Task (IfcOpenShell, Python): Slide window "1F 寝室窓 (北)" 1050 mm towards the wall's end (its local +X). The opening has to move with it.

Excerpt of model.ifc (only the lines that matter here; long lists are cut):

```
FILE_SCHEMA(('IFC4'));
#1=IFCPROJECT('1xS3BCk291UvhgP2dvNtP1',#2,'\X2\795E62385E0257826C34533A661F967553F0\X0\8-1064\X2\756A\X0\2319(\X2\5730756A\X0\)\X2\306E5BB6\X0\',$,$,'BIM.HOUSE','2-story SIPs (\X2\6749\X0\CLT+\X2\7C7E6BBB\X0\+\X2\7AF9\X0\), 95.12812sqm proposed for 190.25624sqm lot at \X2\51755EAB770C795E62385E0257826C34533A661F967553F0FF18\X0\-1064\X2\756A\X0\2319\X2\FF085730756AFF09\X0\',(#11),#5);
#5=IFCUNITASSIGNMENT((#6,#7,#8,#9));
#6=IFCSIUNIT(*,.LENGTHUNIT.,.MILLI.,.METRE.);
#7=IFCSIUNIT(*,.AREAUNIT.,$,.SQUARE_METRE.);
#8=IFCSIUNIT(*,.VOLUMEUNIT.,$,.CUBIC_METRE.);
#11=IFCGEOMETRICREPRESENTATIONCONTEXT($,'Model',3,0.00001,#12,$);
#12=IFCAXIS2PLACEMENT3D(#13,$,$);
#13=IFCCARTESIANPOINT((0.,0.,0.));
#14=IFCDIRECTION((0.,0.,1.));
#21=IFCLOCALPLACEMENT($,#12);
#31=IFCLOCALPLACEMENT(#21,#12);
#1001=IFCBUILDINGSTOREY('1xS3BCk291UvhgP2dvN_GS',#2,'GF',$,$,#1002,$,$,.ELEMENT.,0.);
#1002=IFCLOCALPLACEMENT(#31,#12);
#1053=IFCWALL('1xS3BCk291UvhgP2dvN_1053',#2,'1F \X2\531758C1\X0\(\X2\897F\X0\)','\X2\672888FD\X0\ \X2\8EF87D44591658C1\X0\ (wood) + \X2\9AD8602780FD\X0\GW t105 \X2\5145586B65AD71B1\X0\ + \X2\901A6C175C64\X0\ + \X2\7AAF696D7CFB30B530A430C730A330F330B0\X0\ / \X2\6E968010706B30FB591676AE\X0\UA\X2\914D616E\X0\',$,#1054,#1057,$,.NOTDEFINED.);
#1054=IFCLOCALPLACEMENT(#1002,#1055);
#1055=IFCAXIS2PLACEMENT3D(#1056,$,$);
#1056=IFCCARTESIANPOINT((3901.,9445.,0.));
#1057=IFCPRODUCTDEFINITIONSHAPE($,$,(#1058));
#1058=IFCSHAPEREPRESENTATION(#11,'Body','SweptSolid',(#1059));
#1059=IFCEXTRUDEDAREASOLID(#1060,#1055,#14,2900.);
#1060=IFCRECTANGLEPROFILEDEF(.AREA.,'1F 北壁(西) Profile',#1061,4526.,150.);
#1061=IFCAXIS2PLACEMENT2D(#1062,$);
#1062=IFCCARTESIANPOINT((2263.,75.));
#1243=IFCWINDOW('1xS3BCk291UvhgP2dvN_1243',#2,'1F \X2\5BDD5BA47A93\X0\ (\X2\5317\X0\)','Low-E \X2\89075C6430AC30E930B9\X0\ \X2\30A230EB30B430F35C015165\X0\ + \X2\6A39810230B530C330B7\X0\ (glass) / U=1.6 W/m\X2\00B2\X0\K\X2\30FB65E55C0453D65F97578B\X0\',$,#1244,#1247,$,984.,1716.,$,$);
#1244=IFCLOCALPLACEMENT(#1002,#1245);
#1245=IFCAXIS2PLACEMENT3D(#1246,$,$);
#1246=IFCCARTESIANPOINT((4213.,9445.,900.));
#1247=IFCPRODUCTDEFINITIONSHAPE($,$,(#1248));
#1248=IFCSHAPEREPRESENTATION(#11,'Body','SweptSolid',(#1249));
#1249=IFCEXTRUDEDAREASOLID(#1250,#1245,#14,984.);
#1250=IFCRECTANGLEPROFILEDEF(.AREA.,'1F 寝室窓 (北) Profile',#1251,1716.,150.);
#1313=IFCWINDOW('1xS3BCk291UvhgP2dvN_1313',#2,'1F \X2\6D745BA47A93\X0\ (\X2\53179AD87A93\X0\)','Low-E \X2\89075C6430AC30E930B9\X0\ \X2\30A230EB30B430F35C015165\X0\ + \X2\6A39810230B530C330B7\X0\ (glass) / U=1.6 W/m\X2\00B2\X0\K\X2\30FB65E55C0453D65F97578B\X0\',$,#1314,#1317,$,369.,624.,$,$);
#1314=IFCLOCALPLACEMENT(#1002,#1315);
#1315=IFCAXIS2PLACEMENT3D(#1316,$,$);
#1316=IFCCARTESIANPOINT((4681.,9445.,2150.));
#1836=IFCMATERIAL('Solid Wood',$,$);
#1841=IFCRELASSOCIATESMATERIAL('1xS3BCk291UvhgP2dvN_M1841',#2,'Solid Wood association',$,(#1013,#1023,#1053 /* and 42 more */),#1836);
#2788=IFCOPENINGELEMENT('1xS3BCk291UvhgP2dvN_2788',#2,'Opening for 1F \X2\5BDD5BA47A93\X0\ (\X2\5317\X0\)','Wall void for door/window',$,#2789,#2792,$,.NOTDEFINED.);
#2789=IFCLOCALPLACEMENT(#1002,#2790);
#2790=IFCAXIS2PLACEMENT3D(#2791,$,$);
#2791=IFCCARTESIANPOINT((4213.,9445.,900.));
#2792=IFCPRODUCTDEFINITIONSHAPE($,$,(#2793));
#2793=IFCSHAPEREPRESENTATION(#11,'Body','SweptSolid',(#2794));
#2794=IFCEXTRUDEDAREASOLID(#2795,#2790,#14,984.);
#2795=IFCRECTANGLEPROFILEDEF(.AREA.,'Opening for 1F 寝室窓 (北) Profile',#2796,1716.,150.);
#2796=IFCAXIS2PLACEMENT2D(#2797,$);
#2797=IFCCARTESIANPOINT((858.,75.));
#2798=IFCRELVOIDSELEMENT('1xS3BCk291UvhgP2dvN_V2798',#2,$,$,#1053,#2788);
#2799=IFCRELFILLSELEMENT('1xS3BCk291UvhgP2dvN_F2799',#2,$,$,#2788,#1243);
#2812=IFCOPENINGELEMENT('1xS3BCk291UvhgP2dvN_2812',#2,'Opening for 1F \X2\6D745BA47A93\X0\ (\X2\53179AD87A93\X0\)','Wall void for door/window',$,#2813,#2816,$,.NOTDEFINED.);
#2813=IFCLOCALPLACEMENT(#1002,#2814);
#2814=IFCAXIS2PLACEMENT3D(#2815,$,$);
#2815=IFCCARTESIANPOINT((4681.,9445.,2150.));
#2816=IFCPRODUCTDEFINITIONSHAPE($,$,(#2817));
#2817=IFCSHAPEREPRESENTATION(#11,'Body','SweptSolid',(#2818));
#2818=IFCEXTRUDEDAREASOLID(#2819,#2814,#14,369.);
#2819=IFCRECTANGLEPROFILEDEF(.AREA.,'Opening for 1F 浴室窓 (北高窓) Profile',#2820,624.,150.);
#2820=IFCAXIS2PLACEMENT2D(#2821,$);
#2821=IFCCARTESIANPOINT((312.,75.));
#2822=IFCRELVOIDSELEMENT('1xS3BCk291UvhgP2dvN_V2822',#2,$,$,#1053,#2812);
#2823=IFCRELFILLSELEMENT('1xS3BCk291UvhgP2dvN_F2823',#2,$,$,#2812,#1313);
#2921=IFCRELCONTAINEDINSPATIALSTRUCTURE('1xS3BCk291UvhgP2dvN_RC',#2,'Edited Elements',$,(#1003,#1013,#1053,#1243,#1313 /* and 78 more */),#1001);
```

```python
import ifcopenshell
import ifcopenshell.api.geometry
import ifcopenshell.util.placement
import ifcopenshell.util.unit

model = ifcopenshell.open("model.ifc")
unit_scale = ifcopenshell.util.unit.calculate_unit_scale(model)

window = model.by_guid("1xS3BCk291UvhgP2dvN_1243")
opening = window.FillsVoids[0].RelatingOpeningElement
wall = opening.VoidsElements[0].RelatingBuildingElement

wall_matrix = ifcopenshell.util.placement.get_local_placement(wall.ObjectPlacement)
shift = wall_matrix[:3, 0] * 1.05 / unit_scale
before = ifcopenshell.util.placement.get_local_placement(window.ObjectPlacement)[:3, 3].copy()

# The window is not placed relative to its opening, so move both.
for product in (opening, window):
    matrix = ifcopenshell.util.placement.get_local_placement(product.ObjectPlacement)
    matrix[:3, 3] += shift
    ifcopenshell.api.geometry.edit_object_placement(model, product=product, matrix=matrix, is_si=False)

after = ifcopenshell.util.placement.get_local_placement(window.ObjectPlacement)[:3, 3]
print("window moved by", (after - before).round(3) + 0.0)

model.write("model_edited.ifc")
```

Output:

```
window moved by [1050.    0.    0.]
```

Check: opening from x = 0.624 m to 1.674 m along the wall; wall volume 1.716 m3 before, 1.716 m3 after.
